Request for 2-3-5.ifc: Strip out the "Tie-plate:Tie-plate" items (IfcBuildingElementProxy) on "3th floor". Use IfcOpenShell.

First a look at what the model holds.

```python
import ifcopenshell
import ifcopenshell.util.element

model = ifcopenshell.open("2-3-5.ifc")
print(model.schema)
storey = next(s for s in model.by_type("IfcBuildingStorey") if s.Name == "3th floor")
proxies = [e for e in ifcopenshell.util.element.get_decomposition(storey) if e.is_a("IfcBuildingElementProxy")]
seen = {}
for e in proxies:
    element_type = ifcopenshell.util.element.get_type(e)
    name = element_type.Name if element_type not in (None, e) else None
    seen[name] = seen.get(name, 0) + 1
for name, count in sorted(seen.items(), key=str):
    print(count, "x", name)
```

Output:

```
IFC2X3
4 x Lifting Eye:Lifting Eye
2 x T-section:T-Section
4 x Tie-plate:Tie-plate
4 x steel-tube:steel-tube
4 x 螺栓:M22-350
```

```python
import ifcopenshell
import ifcopenshell.api.root
import ifcopenshell.util.element

model = ifcopenshell.open("2-3-5.ifc")

storey = next(s for s in model.by_type("IfcBuildingStorey") if s.Name == "3th floor")
proxies = [e for e in ifcopenshell.util.element.get_decomposition(storey) if e.is_a("IfcBuildingElementProxy")]
targets = [e for e in proxies if (t := ifcopenshell.util.element.get_type(e)) not in (None, e) and t.Name == "Tie-plate:Tie-plate"]

for e in targets:
    ifcopenshell.api.root.remove_product(model, product=e)
print(len(targets), "removed")

model.write("2-3-5_v2.ifc")
```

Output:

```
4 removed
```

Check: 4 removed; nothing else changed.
